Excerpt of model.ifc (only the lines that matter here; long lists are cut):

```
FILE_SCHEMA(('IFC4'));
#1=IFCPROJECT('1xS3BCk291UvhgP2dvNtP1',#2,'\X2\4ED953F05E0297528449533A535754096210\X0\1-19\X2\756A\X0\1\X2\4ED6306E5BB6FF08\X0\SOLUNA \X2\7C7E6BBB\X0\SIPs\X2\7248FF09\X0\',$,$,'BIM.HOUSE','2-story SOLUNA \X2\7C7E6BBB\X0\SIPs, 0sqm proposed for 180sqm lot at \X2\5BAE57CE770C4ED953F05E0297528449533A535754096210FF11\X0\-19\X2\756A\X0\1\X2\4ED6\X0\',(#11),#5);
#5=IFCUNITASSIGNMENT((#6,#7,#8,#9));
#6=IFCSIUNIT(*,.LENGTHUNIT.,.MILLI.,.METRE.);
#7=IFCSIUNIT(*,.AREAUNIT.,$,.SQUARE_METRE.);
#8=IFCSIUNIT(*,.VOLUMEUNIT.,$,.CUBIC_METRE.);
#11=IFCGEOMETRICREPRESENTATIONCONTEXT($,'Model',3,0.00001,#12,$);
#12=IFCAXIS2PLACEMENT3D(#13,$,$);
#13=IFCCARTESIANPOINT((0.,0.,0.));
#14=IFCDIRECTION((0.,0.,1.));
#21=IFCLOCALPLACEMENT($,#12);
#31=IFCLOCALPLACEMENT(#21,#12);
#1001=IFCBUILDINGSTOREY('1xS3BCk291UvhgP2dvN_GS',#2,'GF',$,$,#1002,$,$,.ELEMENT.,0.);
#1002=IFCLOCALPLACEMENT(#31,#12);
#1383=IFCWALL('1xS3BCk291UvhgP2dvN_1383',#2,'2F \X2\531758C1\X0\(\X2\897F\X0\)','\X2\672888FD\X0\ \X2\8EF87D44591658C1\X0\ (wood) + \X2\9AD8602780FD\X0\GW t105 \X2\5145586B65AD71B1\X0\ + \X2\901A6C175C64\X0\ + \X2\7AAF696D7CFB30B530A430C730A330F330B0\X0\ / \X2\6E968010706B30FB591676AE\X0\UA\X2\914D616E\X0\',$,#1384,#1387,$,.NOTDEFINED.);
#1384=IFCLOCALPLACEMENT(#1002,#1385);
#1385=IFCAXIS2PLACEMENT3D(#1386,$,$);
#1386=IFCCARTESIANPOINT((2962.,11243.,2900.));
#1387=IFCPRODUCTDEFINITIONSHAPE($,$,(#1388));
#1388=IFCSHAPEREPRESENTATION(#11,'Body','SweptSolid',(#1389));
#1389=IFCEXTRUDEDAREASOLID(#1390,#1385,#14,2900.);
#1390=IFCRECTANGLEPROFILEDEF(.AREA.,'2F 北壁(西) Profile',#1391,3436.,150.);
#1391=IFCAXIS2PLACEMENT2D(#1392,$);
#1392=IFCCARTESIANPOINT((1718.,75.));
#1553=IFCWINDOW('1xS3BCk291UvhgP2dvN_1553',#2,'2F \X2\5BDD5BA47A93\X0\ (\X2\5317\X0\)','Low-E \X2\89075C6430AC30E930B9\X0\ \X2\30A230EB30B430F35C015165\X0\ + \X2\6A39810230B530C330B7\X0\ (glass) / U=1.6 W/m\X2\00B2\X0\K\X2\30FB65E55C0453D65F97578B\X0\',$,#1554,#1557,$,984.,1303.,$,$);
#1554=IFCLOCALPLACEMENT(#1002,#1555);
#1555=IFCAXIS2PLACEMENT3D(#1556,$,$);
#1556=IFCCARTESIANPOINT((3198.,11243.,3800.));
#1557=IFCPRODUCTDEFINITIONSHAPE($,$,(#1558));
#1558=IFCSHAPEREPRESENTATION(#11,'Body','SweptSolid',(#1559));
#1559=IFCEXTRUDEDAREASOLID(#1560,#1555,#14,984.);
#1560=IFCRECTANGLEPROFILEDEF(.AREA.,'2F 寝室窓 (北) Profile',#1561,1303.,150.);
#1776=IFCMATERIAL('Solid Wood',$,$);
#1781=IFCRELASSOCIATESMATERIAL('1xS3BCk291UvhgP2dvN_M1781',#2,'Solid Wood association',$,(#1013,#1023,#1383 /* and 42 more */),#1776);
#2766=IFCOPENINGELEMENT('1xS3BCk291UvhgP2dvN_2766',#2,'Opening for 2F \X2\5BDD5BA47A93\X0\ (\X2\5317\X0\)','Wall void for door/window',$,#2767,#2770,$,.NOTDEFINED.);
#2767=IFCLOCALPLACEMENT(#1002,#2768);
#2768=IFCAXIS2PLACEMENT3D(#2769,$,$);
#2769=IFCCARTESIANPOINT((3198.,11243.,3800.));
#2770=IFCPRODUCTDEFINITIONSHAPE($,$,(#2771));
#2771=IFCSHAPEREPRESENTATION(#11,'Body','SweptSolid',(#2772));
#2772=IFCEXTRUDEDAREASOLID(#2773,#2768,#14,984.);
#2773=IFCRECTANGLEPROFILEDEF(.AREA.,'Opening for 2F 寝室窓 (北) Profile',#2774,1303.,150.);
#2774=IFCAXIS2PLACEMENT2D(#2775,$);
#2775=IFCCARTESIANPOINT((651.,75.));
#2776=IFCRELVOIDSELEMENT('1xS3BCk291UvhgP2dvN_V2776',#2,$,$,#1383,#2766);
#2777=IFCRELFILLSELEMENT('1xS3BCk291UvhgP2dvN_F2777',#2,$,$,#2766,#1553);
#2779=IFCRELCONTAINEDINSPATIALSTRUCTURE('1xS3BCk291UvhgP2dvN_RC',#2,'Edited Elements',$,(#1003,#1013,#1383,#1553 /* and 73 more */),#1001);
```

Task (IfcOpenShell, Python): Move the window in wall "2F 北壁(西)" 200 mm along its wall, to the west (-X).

```python
import ifcopenshell
import ifcopenshell.api.geometry
import ifcopenshell.util.placement

model = ifcopenshell.open("model.ifc")

window = model.by_guid("1xS3BCk291UvhgP2dvN_1553")
opening = window.FillsVoids[0].RelatingOpeningElement
wall = opening.VoidsElements[0].RelatingBuildingElement

wall_matrix = ifcopenshell.util.placement.get_local_placement(wall.ObjectPlacement)
shift = wall_matrix[:3, 0] * -200.0
before = ifcopenshell.util.placement.get_local_placement(window.ObjectPlacement)[:3, 3].copy()

# The window is not placed relative to its opening, so move both.
for product in (opening, window):
    matrix = ifcopenshell.util.placement.get_local_placement(product.ObjectPlacement)
    matrix[:3, 3] += shift
    ifcopenshell.api.geometry.edit_object_placement(model, product=product, matrix=matrix, is_si=False)

after = ifcopenshell.util.placement.get_local_placement(window.ObjectPlacement)[:3, 3]
print("window moved by", (after - before).round(3) + 0.0)

model.write("model_v2.ifc")
```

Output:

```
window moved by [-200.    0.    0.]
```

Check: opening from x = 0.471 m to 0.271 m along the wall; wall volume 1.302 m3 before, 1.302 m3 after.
